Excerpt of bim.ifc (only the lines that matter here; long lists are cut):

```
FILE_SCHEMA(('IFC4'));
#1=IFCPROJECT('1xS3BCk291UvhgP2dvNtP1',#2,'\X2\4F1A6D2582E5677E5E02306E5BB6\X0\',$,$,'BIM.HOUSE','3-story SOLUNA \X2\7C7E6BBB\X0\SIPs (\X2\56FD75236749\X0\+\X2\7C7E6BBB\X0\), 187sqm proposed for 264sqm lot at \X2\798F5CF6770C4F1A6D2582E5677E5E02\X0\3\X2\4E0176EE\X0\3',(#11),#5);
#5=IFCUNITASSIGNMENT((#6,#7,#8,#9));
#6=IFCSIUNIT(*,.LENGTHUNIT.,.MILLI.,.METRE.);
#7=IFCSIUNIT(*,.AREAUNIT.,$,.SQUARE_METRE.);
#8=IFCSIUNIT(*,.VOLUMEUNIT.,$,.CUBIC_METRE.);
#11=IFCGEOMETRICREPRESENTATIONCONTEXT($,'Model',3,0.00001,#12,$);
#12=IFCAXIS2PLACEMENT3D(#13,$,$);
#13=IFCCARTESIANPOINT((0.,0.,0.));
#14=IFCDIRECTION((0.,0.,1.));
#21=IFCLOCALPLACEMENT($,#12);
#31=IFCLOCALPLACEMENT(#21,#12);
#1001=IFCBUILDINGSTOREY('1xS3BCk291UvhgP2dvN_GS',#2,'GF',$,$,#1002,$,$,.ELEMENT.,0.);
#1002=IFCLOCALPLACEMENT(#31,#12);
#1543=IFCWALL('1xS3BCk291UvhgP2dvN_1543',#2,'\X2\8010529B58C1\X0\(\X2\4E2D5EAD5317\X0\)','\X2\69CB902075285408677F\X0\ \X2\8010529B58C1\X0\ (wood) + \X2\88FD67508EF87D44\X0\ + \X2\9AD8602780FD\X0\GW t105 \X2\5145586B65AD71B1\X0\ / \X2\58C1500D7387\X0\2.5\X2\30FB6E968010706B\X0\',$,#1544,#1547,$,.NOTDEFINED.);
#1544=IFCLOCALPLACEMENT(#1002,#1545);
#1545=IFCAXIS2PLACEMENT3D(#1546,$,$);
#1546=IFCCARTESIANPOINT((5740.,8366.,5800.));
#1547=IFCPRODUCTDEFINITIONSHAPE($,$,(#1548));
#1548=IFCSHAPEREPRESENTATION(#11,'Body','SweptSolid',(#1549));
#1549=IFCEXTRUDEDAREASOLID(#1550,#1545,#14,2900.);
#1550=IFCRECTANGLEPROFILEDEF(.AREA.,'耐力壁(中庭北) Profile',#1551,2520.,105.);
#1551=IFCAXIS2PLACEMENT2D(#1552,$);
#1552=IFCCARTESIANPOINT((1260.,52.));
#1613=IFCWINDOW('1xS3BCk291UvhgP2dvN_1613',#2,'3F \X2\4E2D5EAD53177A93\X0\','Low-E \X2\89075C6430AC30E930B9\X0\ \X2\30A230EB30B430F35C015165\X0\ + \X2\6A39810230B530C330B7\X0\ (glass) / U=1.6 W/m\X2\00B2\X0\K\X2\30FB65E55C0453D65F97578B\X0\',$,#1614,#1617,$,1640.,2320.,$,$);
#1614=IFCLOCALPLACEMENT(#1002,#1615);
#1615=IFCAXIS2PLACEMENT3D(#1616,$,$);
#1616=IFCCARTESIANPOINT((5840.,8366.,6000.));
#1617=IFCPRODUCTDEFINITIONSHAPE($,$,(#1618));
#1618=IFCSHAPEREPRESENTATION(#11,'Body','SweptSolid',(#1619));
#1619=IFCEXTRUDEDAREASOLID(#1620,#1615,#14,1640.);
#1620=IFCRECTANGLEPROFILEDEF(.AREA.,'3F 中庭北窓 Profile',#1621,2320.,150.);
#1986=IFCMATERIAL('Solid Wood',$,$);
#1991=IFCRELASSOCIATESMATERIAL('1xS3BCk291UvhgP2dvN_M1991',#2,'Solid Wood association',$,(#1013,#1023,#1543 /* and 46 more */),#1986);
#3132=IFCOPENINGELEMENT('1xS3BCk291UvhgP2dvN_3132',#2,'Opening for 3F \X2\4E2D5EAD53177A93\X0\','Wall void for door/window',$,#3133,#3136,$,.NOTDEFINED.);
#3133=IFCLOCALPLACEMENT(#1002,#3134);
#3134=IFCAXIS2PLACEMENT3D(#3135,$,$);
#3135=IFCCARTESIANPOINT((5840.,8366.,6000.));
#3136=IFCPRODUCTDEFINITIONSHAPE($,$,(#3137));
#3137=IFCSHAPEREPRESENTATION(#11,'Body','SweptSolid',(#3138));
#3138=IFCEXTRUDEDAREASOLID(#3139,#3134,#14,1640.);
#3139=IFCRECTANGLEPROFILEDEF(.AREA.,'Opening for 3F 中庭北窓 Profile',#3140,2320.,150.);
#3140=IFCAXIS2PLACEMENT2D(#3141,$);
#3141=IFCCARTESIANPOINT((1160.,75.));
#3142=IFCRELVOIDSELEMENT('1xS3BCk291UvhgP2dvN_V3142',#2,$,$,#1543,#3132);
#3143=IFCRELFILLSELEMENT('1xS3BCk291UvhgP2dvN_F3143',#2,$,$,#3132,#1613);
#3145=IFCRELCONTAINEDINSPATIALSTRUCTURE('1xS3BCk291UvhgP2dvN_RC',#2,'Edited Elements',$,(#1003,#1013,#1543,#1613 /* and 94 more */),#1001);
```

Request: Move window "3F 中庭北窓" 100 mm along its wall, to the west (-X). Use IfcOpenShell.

```python
import ifcopenshell
import ifcopenshell.api.geometry
import ifcopenshell.util.placement
import ifcopenshell.util.unit

model = ifcopenshell.open("bim.ifc")
unit_scale = ifcopenshell.util.unit.calculate_unit_scale(model)

window = model.by_guid("1xS3BCk291UvhgP2dvN_1613")
opening = window.FillsVoids[0].RelatingOpeningElement
wall = opening.VoidsElements[0].RelatingBuildingElement

wall_matrix = ifcopenshell.util.placement.get_local_placement(wall.ObjectPlacement)
shift = wall_matrix[:3, 0] * -0.1 / unit_scale
before = ifcopenshell.util.placement.get_local_placement(window.ObjectPlacement)[:3, 3].copy()

# The window is not placed relative to its opening, so move both.
for product in (opening, window):
    matrix = ifcopenshell.util.placement.get_local_placement(product.ObjectPlacement)
    matrix[:3, 3] += shift
    ifcopenshell.api.geometry.edit_object_placement(model, product=product, matrix=matrix, is_si=False)

after = ifcopenshell.util.placement.get_local_placement(window.ObjectPlacement)[:3, 3]
print("window moved by", (after - before).round(3) + 0.0)

model.write("bim_rev.ifc")
```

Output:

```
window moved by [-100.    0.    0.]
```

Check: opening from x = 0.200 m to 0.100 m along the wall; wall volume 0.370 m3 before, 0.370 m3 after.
